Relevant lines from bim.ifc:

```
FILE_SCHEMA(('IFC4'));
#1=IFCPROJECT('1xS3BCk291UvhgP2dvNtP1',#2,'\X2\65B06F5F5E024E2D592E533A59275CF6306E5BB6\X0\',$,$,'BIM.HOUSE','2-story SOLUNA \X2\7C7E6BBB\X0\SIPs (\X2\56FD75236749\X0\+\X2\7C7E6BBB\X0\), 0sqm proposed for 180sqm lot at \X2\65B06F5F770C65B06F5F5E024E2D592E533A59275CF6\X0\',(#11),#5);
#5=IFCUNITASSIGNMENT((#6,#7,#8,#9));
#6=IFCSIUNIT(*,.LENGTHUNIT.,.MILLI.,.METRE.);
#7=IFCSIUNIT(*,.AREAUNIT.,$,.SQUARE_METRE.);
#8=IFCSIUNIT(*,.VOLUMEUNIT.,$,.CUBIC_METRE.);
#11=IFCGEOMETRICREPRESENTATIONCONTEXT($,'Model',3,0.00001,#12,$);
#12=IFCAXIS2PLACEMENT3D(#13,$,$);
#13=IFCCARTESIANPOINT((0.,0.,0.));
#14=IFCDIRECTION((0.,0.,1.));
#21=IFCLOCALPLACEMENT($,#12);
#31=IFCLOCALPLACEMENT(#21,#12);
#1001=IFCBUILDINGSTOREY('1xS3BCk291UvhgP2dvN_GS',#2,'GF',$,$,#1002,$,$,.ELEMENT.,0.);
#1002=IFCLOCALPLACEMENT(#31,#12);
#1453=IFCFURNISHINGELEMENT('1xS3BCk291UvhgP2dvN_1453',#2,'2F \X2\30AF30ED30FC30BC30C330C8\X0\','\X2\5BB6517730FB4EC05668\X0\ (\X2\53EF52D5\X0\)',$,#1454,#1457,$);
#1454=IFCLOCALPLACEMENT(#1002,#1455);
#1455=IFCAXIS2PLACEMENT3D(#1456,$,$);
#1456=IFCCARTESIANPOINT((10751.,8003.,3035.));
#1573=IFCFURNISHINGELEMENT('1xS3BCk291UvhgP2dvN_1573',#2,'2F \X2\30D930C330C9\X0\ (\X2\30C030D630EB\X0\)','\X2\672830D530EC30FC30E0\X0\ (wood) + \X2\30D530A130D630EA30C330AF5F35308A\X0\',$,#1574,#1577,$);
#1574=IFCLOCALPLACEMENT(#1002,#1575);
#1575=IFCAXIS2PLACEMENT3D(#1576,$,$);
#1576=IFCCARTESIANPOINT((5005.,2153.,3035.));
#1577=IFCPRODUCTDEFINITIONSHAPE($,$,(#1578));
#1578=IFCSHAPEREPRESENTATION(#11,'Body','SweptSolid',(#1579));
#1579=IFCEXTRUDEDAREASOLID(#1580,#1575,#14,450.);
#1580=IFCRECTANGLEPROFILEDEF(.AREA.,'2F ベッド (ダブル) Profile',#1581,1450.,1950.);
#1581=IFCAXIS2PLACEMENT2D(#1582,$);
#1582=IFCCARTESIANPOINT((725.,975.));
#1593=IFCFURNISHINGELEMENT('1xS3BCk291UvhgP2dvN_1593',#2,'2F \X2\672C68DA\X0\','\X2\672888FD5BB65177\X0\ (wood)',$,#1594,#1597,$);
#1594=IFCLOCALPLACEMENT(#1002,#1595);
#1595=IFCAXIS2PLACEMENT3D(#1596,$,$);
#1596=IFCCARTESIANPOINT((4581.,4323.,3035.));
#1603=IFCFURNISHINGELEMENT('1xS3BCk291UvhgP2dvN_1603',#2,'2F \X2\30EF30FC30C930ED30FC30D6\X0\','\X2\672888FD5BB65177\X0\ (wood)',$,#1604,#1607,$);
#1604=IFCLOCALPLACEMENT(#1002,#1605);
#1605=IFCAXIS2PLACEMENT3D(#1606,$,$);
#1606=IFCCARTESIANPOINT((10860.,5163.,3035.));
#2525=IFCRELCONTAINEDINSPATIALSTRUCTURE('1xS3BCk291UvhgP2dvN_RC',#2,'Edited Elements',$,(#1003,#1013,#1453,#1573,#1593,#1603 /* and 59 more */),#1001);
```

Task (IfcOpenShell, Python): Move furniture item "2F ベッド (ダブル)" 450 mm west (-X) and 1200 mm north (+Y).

```python
import ifcopenshell
import ifcopenshell.api.geometry
import ifcopenshell.util.placement
import ifcopenshell.util.unit

model = ifcopenshell.open("bim.ifc")
unit_scale = ifcopenshell.util.unit.calculate_unit_scale(model)

item = model.by_guid("1xS3BCk291UvhgP2dvN_1573")
matrix = ifcopenshell.util.placement.get_local_placement(item.ObjectPlacement)
matrix[0, 3] -= 0.45 / unit_scale
matrix[1, 3] += 1.2 / unit_scale
ifcopenshell.api.geometry.edit_object_placement(model, product=item, matrix=matrix, is_si=False)

print(ifcopenshell.util.placement.get_local_placement(item.ObjectPlacement).round(3) + 0.0)

model.write("bim_rev.ifc")
```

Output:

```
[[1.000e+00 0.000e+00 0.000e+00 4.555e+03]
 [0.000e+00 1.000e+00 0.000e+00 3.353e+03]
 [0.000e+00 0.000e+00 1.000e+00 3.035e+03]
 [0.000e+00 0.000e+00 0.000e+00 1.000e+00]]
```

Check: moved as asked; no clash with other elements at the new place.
